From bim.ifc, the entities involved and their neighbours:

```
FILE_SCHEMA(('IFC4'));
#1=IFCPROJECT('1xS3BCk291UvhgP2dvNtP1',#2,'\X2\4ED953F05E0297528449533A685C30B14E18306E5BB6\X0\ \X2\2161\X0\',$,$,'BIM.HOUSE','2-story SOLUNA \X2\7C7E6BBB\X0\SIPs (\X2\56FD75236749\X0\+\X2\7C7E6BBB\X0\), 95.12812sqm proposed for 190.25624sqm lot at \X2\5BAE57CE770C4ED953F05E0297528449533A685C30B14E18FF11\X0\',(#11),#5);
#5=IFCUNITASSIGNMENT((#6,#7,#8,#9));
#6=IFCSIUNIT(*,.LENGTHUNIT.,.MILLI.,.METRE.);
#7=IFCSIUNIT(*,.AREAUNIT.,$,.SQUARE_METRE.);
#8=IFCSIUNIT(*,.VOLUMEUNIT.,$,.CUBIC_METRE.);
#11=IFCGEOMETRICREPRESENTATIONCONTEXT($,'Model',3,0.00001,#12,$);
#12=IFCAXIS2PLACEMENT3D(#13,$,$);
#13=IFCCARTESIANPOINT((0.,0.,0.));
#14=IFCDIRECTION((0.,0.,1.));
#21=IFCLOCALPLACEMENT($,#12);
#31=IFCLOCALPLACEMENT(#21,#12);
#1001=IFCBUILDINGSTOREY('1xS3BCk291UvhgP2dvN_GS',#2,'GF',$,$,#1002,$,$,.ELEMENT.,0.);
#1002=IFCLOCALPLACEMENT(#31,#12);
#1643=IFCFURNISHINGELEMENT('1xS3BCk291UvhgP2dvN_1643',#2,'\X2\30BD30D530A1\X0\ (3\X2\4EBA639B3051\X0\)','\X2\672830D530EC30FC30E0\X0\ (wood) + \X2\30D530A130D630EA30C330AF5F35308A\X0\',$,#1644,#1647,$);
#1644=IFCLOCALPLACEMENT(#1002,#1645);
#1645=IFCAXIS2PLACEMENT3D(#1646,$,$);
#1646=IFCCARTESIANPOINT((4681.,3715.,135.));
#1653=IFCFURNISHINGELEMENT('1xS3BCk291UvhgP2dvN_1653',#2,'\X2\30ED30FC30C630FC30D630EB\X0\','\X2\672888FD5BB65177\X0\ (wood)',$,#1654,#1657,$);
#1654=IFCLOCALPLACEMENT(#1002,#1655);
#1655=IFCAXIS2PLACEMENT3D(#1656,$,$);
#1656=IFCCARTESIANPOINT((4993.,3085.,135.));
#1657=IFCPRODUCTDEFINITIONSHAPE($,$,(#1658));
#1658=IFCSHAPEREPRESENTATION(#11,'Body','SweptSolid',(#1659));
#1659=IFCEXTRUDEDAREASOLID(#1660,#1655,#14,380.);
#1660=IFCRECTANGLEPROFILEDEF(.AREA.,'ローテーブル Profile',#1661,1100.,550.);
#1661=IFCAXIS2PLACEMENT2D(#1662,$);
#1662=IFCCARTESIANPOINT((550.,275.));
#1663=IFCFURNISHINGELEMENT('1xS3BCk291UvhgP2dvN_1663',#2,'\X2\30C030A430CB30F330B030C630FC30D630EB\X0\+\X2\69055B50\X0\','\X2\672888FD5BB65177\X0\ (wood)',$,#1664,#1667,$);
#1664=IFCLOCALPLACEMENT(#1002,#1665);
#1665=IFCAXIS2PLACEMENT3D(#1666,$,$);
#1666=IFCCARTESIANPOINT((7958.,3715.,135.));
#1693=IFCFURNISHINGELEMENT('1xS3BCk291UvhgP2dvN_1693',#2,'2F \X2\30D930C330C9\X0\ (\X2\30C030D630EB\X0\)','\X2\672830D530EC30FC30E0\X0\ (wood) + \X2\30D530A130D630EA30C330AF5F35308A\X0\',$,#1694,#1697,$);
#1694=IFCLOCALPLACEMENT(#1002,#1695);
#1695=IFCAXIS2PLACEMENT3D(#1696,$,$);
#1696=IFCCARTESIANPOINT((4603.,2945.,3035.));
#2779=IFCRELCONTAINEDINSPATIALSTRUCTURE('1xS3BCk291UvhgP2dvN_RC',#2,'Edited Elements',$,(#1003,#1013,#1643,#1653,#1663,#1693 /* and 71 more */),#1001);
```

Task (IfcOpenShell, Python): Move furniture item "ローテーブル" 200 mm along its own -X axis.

```python
import ifcopenshell
import ifcopenshell.api.geometry
import ifcopenshell.util.placement
import ifcopenshell.util.unit

model = ifcopenshell.open("bim.ifc")
unit_scale = ifcopenshell.util.unit.calculate_unit_scale(model)

item = model.by_guid("1xS3BCk291UvhgP2dvN_1653")
matrix = ifcopenshell.util.placement.get_local_placement(item.ObjectPlacement)
matrix[:3, 3] -= matrix[:3, 0] * 0.2 / unit_scale
ifcopenshell.api.geometry.edit_object_placement(model, product=item, matrix=matrix, is_si=False)

print(ifcopenshell.util.placement.get_local_placement(item.ObjectPlacement).round(3) + 0.0)

model.write("bim-out.ifc")
```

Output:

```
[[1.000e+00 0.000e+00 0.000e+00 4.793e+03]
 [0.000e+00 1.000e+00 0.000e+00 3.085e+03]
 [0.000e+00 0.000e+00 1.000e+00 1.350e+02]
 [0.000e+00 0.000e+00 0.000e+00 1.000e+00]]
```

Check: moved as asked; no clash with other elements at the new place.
